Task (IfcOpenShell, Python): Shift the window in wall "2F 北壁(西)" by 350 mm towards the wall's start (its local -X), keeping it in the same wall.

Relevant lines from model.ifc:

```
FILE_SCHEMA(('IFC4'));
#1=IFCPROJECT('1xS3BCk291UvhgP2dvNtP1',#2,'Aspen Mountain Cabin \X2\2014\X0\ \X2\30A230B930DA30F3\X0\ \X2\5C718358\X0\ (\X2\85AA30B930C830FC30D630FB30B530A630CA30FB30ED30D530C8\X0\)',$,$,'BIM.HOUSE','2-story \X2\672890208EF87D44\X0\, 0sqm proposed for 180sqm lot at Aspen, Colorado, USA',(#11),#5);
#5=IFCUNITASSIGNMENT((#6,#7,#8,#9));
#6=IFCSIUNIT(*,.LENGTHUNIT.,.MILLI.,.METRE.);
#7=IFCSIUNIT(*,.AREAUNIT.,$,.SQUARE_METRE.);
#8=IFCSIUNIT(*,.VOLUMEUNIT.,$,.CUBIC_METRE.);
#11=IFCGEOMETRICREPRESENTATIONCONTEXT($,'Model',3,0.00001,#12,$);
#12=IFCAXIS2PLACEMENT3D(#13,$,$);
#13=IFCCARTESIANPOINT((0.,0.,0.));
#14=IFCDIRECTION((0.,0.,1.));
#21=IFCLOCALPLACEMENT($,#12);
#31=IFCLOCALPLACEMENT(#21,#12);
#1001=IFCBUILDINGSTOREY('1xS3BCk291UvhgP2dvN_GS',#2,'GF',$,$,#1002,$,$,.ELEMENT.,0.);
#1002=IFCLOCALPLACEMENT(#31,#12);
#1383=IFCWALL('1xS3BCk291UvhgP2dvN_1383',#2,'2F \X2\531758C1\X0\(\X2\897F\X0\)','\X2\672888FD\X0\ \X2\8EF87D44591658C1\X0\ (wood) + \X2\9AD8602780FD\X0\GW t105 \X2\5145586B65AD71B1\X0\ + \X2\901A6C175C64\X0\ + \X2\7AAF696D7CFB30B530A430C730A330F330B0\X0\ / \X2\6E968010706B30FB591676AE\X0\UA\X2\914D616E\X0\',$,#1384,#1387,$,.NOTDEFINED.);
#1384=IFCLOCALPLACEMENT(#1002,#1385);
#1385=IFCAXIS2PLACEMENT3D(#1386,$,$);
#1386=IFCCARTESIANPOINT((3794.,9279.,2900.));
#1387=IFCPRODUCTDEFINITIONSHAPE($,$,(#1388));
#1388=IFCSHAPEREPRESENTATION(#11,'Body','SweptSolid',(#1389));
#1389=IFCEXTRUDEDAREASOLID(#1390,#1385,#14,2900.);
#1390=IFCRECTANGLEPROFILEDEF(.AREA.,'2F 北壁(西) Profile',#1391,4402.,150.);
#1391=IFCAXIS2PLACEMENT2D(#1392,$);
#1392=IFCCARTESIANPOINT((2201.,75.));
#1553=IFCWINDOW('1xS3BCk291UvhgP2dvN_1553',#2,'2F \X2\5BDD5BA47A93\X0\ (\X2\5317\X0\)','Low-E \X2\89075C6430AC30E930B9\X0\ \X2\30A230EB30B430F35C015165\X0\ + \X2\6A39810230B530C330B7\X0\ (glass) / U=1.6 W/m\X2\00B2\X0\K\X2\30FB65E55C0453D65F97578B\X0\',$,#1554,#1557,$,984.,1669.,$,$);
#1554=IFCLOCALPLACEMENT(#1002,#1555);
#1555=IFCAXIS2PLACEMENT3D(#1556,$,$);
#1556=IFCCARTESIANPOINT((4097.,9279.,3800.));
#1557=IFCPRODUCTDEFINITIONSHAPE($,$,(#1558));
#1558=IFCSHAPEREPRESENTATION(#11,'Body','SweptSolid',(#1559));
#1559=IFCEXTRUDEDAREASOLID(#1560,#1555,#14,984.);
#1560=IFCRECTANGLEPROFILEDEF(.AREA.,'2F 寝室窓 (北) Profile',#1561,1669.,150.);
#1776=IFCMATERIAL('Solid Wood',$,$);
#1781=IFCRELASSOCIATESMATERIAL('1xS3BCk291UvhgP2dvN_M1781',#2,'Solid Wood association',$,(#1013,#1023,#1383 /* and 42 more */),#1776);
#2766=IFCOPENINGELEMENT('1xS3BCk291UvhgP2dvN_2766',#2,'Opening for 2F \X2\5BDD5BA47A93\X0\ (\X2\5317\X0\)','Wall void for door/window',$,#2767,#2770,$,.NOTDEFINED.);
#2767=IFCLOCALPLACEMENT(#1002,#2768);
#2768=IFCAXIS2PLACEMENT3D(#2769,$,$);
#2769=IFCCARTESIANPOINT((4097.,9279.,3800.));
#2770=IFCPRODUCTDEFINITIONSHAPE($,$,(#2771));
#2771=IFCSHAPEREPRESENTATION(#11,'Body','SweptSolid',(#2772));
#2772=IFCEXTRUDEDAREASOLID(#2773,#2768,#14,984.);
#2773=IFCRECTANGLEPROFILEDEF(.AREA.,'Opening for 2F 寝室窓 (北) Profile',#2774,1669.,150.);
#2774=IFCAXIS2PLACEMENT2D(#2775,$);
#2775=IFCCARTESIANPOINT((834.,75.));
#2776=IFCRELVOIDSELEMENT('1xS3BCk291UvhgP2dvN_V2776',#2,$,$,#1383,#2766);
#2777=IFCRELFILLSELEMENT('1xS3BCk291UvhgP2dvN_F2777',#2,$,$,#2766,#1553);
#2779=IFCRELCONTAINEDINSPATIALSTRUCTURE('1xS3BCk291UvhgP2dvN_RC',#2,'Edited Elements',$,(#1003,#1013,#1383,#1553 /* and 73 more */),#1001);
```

```python
import ifcopenshell
import ifcopenshell.api.geometry
import ifcopenshell.util.placement
import ifcopenshell.util.unit

model = ifcopenshell.open("model.ifc")
unit_scale = ifcopenshell.util.unit.calculate_unit_scale(model)

window = model.by_guid("1xS3BCk291UvhgP2dvN_1553")
opening = window.FillsVoids[0].RelatingOpeningElement
wall = opening.VoidsElements[0].RelatingBuildingElement

wall_matrix = ifcopenshell.util.placement.get_local_placement(wall.ObjectPlacement)
shift = wall_matrix[:3, 0] * -0.35 / unit_scale
before = ifcopenshell.util.placement.get_local_placement(window.ObjectPlacement)[:3, 3].copy()

# The window is not placed relative to its opening, so move both.
for product in (opening, window):
    matrix = ifcopenshell.util.placement.get_local_placement(product.ObjectPlacement)
    matrix[:3, 3] += shift
    ifcopenshell.api.geometry.edit_object_placement(model, product=product, matrix=matrix, is_si=False)

after = ifcopenshell.util.placement.get_local_placement(window.ObjectPlacement)[:3, 3]
print("window moved by", (after - before).round(3) + 0.0)

model.write("model_edited.ifc")
```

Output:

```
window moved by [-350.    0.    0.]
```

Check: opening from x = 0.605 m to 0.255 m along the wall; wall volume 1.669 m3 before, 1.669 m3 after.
